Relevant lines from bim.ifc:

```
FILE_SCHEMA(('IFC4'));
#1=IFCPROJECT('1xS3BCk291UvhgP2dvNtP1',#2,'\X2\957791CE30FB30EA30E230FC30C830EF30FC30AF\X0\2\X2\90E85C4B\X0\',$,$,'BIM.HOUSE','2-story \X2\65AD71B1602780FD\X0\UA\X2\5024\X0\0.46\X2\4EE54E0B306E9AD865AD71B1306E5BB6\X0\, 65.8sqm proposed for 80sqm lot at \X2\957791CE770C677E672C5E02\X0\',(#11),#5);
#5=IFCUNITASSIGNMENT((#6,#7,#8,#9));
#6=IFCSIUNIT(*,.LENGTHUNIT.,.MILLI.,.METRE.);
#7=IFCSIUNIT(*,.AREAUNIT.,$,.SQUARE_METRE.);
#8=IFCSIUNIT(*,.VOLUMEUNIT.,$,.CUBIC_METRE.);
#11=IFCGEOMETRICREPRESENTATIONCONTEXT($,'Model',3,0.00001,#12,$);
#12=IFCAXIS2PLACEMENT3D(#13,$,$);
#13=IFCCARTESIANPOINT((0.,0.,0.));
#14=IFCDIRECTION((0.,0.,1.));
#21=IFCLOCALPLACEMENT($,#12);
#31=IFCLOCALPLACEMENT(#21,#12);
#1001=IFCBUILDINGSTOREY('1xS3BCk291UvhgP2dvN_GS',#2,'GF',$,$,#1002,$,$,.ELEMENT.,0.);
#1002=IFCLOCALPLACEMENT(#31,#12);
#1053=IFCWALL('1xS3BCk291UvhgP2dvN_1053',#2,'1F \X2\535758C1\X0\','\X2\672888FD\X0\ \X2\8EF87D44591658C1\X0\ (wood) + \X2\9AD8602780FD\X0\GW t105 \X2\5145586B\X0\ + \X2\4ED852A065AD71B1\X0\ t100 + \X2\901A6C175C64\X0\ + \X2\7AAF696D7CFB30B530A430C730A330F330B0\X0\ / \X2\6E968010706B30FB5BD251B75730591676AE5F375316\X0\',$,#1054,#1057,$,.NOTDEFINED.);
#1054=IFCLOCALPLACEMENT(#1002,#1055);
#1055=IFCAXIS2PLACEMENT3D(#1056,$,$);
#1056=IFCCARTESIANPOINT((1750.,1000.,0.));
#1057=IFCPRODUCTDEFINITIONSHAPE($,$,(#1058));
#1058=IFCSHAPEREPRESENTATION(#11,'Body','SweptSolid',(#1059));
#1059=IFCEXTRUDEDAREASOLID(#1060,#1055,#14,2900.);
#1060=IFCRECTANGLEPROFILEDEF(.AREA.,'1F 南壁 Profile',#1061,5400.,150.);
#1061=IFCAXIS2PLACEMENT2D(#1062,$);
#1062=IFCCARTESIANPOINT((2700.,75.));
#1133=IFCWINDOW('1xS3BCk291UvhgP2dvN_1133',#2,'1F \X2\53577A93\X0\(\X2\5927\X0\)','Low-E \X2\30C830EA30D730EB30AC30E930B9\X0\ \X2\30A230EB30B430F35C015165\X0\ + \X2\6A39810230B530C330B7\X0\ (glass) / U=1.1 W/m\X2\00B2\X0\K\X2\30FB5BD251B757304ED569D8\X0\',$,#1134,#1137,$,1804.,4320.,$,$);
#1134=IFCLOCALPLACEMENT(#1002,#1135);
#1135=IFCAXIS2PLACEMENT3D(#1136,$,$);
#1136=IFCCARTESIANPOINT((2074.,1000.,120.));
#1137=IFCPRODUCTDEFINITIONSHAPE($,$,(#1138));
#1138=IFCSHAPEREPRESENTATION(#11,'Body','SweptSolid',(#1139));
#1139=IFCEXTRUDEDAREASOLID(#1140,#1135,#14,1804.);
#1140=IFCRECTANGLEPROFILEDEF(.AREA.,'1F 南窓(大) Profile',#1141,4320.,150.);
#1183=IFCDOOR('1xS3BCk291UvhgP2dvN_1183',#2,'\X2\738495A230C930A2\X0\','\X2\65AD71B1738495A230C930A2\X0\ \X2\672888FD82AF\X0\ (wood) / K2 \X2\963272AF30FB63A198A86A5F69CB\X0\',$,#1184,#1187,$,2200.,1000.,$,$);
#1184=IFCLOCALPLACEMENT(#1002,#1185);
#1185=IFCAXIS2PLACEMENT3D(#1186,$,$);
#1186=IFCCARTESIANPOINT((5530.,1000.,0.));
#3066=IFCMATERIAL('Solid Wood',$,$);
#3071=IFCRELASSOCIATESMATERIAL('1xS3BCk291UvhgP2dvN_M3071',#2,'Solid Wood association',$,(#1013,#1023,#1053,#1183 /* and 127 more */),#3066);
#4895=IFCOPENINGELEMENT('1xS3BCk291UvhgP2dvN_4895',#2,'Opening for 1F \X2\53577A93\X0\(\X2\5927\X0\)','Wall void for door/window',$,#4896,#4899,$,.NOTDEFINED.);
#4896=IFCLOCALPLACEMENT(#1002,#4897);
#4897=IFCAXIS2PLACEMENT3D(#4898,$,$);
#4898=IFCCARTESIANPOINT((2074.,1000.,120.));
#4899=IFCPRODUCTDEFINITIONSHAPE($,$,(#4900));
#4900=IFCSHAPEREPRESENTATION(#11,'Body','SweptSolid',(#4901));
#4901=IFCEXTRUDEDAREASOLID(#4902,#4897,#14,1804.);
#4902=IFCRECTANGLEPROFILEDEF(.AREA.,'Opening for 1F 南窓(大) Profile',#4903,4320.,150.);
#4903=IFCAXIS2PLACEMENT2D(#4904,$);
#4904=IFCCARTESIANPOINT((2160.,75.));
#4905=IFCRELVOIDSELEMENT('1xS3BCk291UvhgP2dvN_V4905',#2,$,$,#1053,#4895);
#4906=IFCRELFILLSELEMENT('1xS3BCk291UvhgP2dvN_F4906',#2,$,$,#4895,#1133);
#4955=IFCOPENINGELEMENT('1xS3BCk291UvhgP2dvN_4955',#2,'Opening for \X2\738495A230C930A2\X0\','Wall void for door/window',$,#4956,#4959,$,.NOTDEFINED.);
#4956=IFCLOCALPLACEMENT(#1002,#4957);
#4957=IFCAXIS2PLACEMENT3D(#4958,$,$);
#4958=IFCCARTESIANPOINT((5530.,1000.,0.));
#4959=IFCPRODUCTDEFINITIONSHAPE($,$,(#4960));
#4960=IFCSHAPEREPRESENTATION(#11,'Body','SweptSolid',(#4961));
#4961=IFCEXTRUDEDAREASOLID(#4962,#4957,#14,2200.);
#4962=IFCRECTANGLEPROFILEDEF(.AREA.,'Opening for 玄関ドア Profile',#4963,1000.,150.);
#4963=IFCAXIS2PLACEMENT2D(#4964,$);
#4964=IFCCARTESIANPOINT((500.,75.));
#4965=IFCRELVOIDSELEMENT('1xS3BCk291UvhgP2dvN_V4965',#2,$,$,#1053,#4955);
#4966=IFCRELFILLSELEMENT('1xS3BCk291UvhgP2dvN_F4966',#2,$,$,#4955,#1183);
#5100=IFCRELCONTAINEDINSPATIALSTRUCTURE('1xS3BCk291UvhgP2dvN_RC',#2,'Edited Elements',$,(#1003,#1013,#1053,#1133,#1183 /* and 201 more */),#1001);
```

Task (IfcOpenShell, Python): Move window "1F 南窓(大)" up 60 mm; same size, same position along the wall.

```python
import numpy as np
import ifcopenshell
import ifcopenshell.api.geometry
import ifcopenshell.util.placement
import ifcopenshell.util.unit

model = ifcopenshell.open("bim.ifc")
unit_scale = ifcopenshell.util.unit.calculate_unit_scale(model)

window = model.by_guid("1xS3BCk291UvhgP2dvN_1133")
opening = window.FillsVoids[0].RelatingOpeningElement
dz = 0.06 / unit_scale

shift = np.array([0.0, 0.0, dz])
# The window is not placed relative to its opening, so move both.
for product in (opening, window):
    matrix = ifcopenshell.util.placement.get_local_placement(product.ObjectPlacement)
    matrix[:3, 3] += shift
    ifcopenshell.api.geometry.edit_object_placement(model, product=product, matrix=matrix, is_si=False)

print(f"moved by {dz * unit_scale:+.3f} m")

model.write("bim_rev.ifc")
```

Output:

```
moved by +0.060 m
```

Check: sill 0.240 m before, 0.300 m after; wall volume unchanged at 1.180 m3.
